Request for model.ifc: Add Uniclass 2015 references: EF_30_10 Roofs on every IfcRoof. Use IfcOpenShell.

First a look at what the model holds.

```python
import ifcopenshell

model = ifcopenshell.open("model.ifc")
print(model.schema)
print("classifications:", [c.Name for c in model.by_type("IfcClassification")])
for ifc_class in ("IfcDoor", "IfcRoof", "IfcStair", "IfcWall", "IfcWindow"):
    print(ifc_class, len(model.by_type(ifc_class)))
```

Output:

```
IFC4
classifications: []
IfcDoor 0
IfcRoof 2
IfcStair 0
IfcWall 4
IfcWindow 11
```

```python
import ifcopenshell
import ifcopenshell.api.classification

model = ifcopenshell.open("model.ifc")

system = ifcopenshell.api.classification.add_classification(model, classification="Uniclass 2015")

codes = {
    "IfcRoof": ("EF_30_10", "Roofs"),
}
for ifc_class, (code, name) in codes.items():
    products = model.by_type(ifc_class)
    ifcopenshell.api.classification.add_reference(
        model, products=products, classification=system, identification=code, name=name
    )
    print(code, len(products))

model.write("model_edited.ifc")
```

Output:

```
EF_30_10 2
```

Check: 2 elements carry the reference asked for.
